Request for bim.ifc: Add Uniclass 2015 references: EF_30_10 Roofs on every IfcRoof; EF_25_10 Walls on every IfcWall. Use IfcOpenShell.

First a look at what the model holds.

```python
import ifcopenshell

model = ifcopenshell.open("bim.ifc")
print(model.schema)
print("classifications:", [c.Name for c in model.by_type("IfcClassification")])
for ifc_class in ("IfcDoor", "IfcRoof", "IfcStair", "IfcWall", "IfcWindow"):
    print(ifc_class, len(model.by_type(ifc_class)))
```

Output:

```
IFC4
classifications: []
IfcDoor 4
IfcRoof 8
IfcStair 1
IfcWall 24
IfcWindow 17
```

```python
import ifcopenshell
import ifcopenshell.api.classification

model = ifcopenshell.open("bim.ifc")

system = ifcopenshell.api.classification.add_classification(model, classification="Uniclass 2015")

codes = {
    "IfcRoof": ("EF_30_10", "Roofs"),
    "IfcWall": ("EF_25_10", "Walls"),
}
for ifc_class, (code, name) in codes.items():
    products = model.by_type(ifc_class)
    ifcopenshell.api.classification.add_reference(
        model, products=products, classification=system, identification=code, name=name
    )
    print(code, len(products))

model.write("bim_v2.ifc")
```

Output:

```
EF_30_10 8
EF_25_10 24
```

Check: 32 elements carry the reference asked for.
